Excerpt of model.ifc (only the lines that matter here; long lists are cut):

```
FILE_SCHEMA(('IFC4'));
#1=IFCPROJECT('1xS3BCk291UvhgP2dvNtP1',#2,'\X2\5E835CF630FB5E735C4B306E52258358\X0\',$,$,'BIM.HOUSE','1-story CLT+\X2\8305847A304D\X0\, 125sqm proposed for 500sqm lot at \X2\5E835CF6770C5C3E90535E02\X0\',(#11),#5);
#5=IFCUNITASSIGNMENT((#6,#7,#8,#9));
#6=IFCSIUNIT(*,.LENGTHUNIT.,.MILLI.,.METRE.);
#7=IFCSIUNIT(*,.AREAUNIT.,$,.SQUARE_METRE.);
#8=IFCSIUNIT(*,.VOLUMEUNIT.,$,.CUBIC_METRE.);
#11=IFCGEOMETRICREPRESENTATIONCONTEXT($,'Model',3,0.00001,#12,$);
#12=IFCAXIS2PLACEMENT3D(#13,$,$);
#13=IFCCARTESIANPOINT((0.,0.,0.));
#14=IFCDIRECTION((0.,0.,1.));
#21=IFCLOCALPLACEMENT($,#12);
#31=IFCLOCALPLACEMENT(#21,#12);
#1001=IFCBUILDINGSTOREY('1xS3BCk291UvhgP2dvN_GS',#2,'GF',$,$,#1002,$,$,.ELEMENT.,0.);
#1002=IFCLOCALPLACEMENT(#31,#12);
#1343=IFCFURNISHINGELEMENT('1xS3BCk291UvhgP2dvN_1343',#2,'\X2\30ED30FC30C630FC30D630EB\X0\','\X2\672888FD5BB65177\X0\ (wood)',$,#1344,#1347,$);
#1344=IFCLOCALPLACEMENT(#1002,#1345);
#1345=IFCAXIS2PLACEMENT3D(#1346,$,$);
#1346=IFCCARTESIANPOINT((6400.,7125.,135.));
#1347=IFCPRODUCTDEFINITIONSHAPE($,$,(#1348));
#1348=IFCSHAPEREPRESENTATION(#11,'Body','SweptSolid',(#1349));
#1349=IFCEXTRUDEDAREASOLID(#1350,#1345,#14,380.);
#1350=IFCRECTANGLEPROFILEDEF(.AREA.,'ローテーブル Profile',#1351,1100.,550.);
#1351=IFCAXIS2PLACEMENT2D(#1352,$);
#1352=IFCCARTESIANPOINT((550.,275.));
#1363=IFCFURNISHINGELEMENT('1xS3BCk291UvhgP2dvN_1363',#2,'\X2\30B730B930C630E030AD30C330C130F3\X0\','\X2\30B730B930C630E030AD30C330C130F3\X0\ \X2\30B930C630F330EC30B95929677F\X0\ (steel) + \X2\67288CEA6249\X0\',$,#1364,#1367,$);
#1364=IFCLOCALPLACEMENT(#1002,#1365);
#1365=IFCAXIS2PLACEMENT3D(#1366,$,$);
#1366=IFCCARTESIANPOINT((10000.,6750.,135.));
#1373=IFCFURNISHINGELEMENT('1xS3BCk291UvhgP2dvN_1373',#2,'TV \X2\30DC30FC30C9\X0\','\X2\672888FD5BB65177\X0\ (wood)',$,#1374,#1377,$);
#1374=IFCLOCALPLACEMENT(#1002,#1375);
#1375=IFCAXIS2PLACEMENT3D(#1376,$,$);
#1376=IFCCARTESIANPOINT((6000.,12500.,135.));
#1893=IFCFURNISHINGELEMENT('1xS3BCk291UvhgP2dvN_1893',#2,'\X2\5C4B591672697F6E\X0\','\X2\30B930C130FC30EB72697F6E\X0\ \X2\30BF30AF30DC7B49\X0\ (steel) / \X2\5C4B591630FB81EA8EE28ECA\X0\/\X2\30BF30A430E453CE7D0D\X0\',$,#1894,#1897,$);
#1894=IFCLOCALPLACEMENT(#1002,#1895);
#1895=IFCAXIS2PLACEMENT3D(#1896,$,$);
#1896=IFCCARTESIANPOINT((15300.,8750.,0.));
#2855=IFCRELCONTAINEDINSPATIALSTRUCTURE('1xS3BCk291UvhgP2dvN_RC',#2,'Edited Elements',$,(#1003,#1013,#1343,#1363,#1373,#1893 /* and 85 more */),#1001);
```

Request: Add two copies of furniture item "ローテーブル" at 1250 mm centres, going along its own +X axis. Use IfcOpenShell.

```python
import ifcopenshell
import ifcopenshell.api.geometry
import ifcopenshell.api.root
import ifcopenshell.util.element
import ifcopenshell.util.placement
import ifcopenshell.util.unit

model = ifcopenshell.open("model.ifc")
unit_scale = ifcopenshell.util.unit.calculate_unit_scale(model)


def reuse_history(source, copy):
    """copy_class also copies each property set's owner history, people and application; keep the originals."""
    for rel in copy.IsDefinedBy:
        if rel.is_a("IfcRelDefinesByProperties") and (history := rel.RelatingPropertyDefinition.OwnerHistory):
            rel.RelatingPropertyDefinition.OwnerHistory = source.OwnerHistory
            ifcopenshell.util.element.remove_deep2(model, history)


source = model.by_id(1343)
base = ifcopenshell.util.placement.get_local_placement(source.ObjectPlacement)
step = base[:3, 0] * 1.25 / unit_scale

for i in range(1, 3):
    copy = ifcopenshell.api.root.copy_class(model, product=source)
    copy.Representation = ifcopenshell.util.element.copy_deep(
        model, source.Representation, exclude=["IfcGeometricRepresentationContext", "IfcRepresentationMap"]
    )
    reuse_history(source, copy)
    matrix = base.copy()
    matrix[:3, 3] += i * step
    print("added at", matrix[:3, 3].round(3) + 0.0)
    ifcopenshell.api.geometry.edit_object_placement(model, product=copy, matrix=matrix, is_si=False)

model.write("model_edited.ifc")
```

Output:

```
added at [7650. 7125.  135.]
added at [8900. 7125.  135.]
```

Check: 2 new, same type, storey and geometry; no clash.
